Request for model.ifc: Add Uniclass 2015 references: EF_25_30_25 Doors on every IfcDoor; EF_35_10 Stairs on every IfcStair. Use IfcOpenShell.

First a look at what the model holds.

```python
import ifcopenshell

model = ifcopenshell.open("model.ifc")
print(model.schema)
print("classifications:", [c.Name for c in model.by_type("IfcClassification")])
for ifc_class in ("IfcDoor", "IfcRoof", "IfcStair", "IfcWall", "IfcWindow"):
    print(ifc_class, len(model.by_type(ifc_class)))
```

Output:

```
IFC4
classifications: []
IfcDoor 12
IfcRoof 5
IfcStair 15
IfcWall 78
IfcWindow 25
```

```python
import ifcopenshell
import ifcopenshell.api.classification

model = ifcopenshell.open("model.ifc")

system = ifcopenshell.api.classification.add_classification(model, classification="Uniclass 2015")

codes = {
    "IfcDoor": ("EF_25_30_25", "Doors"),
    "IfcStair": ("EF_35_10", "Stairs"),
}
for ifc_class, (code, name) in codes.items():
    products = model.by_type(ifc_class)
    ifcopenshell.api.classification.add_reference(
        model, products=products, classification=system, identification=code, name=name
    )
    print(code, len(products))

model.write("model_rev.ifc")
```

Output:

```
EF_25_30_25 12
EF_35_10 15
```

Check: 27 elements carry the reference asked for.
